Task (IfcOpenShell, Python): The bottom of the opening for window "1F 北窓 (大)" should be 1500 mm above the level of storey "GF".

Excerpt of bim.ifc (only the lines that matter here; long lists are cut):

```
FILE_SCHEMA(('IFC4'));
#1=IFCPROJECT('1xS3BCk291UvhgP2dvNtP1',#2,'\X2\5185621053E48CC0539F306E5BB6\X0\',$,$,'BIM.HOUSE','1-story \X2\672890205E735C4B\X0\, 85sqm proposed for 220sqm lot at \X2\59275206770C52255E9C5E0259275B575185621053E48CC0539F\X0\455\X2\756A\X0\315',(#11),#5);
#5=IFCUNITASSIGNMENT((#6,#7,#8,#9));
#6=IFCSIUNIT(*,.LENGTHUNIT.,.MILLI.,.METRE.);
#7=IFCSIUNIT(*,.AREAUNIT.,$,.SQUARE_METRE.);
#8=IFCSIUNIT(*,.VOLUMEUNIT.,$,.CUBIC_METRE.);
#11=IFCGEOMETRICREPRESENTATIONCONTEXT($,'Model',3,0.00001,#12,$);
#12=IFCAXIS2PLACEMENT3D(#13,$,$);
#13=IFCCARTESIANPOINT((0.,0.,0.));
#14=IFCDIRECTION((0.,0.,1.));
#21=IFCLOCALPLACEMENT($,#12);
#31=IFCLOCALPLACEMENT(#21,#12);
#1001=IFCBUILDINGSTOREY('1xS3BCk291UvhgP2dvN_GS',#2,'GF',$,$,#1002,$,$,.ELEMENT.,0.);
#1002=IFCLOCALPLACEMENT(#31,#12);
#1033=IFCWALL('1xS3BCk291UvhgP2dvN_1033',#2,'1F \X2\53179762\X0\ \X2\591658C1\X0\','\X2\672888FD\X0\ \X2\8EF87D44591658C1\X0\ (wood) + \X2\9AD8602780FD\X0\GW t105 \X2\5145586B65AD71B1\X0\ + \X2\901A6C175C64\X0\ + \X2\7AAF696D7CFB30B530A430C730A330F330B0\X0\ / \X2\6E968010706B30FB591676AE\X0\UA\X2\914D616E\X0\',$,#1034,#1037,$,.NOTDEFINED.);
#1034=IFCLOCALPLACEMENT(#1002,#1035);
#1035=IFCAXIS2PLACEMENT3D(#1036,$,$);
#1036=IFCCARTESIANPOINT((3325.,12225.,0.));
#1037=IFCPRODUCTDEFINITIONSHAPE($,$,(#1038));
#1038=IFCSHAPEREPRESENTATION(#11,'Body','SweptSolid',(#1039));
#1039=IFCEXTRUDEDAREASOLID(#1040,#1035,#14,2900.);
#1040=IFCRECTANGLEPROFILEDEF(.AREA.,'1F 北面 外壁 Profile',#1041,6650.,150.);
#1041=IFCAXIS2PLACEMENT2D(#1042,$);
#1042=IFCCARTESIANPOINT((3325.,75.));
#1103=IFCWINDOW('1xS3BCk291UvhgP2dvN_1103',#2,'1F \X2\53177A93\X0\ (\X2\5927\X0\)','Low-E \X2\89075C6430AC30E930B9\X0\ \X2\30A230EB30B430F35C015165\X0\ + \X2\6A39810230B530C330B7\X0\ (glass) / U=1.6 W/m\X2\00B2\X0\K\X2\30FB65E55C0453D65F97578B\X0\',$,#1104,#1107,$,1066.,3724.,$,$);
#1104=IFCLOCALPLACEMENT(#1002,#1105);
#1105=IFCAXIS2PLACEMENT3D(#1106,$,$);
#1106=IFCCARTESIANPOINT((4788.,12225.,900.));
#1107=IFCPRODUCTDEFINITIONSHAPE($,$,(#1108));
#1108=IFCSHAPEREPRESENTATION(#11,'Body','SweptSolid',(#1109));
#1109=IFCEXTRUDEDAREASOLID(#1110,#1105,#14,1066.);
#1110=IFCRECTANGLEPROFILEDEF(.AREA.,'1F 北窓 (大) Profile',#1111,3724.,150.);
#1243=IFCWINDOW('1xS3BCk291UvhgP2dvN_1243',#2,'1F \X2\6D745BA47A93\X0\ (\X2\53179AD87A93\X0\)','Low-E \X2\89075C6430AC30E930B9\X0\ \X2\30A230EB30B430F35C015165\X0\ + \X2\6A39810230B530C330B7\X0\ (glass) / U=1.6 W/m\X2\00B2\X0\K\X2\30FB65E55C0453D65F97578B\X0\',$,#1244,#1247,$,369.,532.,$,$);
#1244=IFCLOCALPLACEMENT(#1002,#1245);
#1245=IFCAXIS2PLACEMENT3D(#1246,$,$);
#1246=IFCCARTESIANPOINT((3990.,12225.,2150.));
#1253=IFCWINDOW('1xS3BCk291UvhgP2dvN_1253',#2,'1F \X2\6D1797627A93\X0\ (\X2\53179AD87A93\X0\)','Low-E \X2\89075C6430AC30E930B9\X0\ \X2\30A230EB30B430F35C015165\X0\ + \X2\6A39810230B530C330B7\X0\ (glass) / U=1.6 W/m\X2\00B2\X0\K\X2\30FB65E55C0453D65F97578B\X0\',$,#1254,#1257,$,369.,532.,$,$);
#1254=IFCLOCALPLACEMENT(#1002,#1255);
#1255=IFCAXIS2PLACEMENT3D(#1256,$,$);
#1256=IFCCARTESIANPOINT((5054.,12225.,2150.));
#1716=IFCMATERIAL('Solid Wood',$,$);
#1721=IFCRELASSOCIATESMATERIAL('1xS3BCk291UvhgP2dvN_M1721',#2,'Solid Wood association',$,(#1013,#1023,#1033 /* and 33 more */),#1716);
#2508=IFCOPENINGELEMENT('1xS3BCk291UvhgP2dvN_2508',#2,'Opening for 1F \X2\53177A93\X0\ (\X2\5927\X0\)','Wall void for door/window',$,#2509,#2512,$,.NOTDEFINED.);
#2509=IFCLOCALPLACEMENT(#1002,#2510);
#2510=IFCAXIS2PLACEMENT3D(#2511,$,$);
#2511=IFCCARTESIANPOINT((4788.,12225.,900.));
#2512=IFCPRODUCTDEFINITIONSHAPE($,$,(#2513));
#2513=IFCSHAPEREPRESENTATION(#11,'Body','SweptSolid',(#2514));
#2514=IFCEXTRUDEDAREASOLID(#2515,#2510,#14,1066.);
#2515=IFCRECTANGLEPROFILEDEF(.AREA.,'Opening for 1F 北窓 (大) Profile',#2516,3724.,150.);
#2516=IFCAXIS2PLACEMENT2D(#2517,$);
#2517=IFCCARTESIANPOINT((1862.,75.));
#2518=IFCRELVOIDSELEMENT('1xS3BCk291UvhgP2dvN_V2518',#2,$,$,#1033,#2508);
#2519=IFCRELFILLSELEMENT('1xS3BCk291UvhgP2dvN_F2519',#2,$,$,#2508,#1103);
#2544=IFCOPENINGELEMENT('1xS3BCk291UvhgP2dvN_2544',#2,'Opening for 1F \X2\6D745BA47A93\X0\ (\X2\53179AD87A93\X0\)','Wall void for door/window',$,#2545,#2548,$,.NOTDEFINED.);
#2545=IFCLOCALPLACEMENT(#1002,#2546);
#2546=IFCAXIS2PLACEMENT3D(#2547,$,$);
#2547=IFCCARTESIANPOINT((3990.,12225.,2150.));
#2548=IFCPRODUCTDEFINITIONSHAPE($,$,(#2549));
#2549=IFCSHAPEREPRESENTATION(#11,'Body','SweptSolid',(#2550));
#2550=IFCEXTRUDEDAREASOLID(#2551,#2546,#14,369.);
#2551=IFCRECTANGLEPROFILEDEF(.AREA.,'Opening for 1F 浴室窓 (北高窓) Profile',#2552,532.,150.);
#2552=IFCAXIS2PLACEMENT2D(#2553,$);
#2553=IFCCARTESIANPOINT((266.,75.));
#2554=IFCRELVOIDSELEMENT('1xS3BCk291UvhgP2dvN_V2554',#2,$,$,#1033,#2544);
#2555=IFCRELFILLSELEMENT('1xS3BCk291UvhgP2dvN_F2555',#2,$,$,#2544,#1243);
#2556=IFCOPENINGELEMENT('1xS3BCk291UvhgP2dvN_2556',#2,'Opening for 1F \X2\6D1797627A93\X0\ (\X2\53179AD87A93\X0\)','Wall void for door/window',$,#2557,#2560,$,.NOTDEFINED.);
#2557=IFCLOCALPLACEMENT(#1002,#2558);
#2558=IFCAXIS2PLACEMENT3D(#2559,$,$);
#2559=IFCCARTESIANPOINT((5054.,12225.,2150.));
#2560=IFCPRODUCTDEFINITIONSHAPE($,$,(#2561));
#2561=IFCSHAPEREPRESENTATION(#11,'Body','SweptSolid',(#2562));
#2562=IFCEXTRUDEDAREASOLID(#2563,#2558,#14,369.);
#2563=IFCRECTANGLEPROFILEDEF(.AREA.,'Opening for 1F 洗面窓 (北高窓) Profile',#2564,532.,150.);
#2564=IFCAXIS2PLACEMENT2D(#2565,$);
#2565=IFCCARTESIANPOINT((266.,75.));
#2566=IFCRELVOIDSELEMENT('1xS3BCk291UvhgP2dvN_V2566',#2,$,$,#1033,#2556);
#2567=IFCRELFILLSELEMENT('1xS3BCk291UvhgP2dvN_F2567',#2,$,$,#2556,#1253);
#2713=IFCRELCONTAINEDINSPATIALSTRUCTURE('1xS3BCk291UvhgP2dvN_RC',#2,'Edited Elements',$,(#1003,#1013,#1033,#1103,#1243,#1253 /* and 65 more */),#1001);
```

```python
import numpy as np
import ifcopenshell
import ifcopenshell.api.geometry
import ifcopenshell.geom
import ifcopenshell.util.element
import ifcopenshell.util.placement
import ifcopenshell.util.shape
import ifcopenshell.util.unit

model = ifcopenshell.open("bim.ifc")
unit_scale = ifcopenshell.util.unit.calculate_unit_scale(model)

window = model.by_id(1103)
opening = window.FillsVoids[0].RelatingOpeningElement
storey = ifcopenshell.util.element.get_container(window, ifc_class="IfcBuildingStorey")
level = ifcopenshell.util.placement.get_local_placement(storey.ObjectPlacement)[2, 3]

# The opening's origin need not be at the sill, so measure its lowest point.
shape = ifcopenshell.geom.create_shape(ifcopenshell.geom.settings(), opening)
bottom = ifcopenshell.util.shape.get_shape_bottom_elevation(shape, shape.geometry) / unit_scale
dz = level + 1.5 / unit_scale - bottom

shift = np.array([0.0, 0.0, dz])
# The window is not placed relative to its opening, so move both.
for product in (opening, window):
    matrix = ifcopenshell.util.placement.get_local_placement(product.ObjectPlacement)
    matrix[:3, 3] += shift
    ifcopenshell.api.geometry.edit_object_placement(model, product=product, matrix=matrix, is_si=False)

print(f"moved by {dz * unit_scale:+.3f} m")

model.write("bim_v2.ifc")
```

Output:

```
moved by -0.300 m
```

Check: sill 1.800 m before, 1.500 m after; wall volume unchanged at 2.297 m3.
